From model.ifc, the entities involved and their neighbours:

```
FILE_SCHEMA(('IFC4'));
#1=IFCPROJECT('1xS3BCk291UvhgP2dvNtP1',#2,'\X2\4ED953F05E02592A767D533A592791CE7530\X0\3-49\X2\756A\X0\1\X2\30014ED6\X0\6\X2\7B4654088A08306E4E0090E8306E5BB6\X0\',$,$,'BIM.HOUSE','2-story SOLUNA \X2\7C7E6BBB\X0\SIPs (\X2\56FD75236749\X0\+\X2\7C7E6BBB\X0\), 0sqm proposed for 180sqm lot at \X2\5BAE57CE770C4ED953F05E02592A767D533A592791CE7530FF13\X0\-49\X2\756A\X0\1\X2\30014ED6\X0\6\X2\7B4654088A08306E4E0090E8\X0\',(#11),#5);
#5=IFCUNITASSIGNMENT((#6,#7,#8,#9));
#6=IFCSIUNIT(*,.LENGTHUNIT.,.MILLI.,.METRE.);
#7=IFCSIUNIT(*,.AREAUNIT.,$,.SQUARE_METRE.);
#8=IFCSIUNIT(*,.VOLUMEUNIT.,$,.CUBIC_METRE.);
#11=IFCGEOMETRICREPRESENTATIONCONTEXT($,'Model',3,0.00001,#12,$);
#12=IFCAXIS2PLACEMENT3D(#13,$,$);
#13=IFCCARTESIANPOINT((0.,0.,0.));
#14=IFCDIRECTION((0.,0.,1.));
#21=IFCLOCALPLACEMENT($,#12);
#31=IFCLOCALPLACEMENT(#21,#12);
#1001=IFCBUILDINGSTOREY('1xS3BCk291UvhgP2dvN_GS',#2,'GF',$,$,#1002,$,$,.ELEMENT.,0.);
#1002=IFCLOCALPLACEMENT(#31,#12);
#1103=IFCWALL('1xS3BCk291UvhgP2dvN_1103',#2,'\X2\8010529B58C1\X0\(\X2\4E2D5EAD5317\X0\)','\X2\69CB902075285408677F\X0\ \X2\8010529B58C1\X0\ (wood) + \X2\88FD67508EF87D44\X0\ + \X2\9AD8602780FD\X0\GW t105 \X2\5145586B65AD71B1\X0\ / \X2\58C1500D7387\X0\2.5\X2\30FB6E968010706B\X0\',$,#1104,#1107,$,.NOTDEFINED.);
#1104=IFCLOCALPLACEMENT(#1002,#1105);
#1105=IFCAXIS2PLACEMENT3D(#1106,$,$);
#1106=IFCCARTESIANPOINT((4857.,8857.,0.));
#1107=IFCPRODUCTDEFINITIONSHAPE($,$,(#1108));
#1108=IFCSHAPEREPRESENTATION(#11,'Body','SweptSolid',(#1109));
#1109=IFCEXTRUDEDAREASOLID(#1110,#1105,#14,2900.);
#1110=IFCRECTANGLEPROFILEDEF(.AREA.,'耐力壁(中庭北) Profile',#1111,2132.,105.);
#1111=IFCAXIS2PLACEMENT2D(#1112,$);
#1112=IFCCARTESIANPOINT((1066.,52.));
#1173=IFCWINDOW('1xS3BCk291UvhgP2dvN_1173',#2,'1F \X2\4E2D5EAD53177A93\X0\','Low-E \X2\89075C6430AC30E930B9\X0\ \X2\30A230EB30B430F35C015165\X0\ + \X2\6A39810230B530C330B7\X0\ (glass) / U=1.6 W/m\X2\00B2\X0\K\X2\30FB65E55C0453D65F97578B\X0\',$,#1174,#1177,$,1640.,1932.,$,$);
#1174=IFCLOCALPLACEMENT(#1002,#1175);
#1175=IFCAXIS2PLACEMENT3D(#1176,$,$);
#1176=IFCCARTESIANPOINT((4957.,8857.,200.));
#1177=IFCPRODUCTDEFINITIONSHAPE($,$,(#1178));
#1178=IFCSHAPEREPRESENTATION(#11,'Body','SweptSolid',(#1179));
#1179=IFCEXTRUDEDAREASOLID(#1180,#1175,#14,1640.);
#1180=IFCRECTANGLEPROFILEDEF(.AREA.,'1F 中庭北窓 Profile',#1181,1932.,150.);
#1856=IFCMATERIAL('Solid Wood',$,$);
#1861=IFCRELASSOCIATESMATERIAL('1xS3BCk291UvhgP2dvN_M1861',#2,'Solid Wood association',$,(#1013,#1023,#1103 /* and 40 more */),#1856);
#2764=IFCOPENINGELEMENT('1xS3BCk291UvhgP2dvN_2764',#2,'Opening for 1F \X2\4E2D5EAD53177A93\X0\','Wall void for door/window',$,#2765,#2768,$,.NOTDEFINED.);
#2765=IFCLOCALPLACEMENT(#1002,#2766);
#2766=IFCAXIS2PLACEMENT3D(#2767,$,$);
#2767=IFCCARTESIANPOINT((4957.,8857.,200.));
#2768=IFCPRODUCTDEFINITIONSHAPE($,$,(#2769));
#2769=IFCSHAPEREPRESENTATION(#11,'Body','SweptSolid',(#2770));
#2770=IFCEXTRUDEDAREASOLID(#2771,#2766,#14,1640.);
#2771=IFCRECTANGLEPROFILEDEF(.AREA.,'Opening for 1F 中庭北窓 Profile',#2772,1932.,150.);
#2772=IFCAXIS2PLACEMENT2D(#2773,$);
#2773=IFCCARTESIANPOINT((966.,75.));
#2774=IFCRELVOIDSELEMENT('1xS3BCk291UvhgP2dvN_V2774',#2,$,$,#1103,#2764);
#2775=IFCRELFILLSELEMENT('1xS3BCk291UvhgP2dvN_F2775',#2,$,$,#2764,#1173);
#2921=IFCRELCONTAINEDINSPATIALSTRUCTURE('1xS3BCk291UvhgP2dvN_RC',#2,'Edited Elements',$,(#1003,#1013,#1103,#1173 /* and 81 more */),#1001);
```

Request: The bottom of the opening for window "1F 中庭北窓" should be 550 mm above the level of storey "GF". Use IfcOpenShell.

```python
import numpy as np
import ifcopenshell
import ifcopenshell.api.geometry
import ifcopenshell.geom
import ifcopenshell.util.element
import ifcopenshell.util.placement
import ifcopenshell.util.shape
import ifcopenshell.util.unit

model = ifcopenshell.open("model.ifc")
unit_scale = ifcopenshell.util.unit.calculate_unit_scale(model)

window = model.by_guid("1xS3BCk291UvhgP2dvN_1173")
opening = window.FillsVoids[0].RelatingOpeningElement
storey = ifcopenshell.util.element.get_container(window, ifc_class="IfcBuildingStorey")
level = ifcopenshell.util.placement.get_local_placement(storey.ObjectPlacement)[2, 3]

# The opening's origin need not be at the sill, so measure its lowest point.
shape = ifcopenshell.geom.create_shape(ifcopenshell.geom.settings(), opening)
bottom = ifcopenshell.util.shape.get_shape_bottom_elevation(shape, shape.geometry) / unit_scale
dz = level + 550.0 - bottom

shift = np.array([0.0, 0.0, dz])
# The window is not placed relative to its opening, so move both.
for product in (opening, window):
    matrix = ifcopenshell.util.placement.get_local_placement(product.ObjectPlacement)
    matrix[:3, 3] += shift
    ifcopenshell.api.geometry.edit_object_placement(model, product=product, matrix=matrix, is_si=False)

print(f"moved by {dz * unit_scale:+.3f} m")

model.write("model_updated.ifc")
```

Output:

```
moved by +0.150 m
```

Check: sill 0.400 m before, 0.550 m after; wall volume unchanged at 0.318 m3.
